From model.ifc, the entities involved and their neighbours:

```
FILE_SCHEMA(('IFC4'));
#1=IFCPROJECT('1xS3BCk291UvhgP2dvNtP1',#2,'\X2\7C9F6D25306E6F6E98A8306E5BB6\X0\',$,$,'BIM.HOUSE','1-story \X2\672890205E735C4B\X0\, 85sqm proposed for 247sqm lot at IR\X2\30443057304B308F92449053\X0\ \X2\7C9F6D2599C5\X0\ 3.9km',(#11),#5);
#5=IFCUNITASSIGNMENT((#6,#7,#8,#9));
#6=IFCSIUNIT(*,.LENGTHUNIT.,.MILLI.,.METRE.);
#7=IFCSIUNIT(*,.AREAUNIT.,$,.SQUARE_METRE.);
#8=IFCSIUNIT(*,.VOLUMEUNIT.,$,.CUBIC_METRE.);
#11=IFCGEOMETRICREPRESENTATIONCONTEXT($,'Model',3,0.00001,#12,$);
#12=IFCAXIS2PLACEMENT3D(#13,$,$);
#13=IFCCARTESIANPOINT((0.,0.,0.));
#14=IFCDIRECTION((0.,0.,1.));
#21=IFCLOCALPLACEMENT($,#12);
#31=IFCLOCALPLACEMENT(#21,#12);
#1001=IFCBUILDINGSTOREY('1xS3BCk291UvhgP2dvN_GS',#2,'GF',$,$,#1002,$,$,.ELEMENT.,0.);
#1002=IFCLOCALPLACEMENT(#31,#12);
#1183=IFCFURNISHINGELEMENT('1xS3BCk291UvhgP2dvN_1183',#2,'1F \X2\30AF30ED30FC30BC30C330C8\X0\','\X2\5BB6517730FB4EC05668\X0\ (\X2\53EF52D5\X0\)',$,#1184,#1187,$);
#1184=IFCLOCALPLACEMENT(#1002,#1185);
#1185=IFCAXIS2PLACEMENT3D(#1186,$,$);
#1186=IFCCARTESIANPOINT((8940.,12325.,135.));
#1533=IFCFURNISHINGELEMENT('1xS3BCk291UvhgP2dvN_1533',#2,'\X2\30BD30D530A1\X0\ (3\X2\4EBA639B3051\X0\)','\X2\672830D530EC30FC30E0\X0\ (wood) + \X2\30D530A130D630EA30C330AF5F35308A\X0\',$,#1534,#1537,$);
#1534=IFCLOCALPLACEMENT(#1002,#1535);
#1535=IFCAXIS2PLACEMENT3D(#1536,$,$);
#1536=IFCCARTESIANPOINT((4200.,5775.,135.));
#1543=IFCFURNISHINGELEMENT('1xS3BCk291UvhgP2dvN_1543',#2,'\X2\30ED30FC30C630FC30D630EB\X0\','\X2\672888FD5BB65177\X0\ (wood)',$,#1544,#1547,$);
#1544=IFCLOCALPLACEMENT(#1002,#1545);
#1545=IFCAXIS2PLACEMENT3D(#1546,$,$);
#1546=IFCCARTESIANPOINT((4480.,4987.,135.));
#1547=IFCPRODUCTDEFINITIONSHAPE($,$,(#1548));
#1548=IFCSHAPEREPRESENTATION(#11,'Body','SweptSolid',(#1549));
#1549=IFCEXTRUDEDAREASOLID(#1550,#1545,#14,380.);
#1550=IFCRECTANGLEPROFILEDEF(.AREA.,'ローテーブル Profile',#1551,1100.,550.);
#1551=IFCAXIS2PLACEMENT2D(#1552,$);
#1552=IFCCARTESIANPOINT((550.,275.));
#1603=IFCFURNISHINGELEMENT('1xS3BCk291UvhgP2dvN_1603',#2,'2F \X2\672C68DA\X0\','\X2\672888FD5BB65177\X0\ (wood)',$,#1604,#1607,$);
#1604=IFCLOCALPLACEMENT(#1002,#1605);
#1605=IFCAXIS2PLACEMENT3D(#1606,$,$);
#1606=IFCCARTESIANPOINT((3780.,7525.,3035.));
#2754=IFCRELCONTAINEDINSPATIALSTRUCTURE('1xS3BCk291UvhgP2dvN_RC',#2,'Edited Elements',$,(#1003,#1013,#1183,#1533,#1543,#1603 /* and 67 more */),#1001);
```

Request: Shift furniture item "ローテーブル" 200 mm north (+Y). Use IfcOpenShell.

```python
import ifcopenshell
import ifcopenshell.api.geometry
import ifcopenshell.util.placement
import ifcopenshell.util.unit

model = ifcopenshell.open("model.ifc")
unit_scale = ifcopenshell.util.unit.calculate_unit_scale(model)

item = model.by_guid("1xS3BCk291UvhgP2dvN_1543")
matrix = ifcopenshell.util.placement.get_local_placement(item.ObjectPlacement)
matrix[1, 3] += 0.2 / unit_scale
ifcopenshell.api.geometry.edit_object_placement(model, product=item, matrix=matrix, is_si=False)

print(ifcopenshell.util.placement.get_local_placement(item.ObjectPlacement).round(3) + 0.0)

model.write("model_v2.ifc")
```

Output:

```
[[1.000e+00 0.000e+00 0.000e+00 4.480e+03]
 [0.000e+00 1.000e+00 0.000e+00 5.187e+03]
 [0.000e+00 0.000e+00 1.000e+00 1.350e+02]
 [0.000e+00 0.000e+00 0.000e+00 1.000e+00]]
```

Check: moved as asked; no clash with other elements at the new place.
